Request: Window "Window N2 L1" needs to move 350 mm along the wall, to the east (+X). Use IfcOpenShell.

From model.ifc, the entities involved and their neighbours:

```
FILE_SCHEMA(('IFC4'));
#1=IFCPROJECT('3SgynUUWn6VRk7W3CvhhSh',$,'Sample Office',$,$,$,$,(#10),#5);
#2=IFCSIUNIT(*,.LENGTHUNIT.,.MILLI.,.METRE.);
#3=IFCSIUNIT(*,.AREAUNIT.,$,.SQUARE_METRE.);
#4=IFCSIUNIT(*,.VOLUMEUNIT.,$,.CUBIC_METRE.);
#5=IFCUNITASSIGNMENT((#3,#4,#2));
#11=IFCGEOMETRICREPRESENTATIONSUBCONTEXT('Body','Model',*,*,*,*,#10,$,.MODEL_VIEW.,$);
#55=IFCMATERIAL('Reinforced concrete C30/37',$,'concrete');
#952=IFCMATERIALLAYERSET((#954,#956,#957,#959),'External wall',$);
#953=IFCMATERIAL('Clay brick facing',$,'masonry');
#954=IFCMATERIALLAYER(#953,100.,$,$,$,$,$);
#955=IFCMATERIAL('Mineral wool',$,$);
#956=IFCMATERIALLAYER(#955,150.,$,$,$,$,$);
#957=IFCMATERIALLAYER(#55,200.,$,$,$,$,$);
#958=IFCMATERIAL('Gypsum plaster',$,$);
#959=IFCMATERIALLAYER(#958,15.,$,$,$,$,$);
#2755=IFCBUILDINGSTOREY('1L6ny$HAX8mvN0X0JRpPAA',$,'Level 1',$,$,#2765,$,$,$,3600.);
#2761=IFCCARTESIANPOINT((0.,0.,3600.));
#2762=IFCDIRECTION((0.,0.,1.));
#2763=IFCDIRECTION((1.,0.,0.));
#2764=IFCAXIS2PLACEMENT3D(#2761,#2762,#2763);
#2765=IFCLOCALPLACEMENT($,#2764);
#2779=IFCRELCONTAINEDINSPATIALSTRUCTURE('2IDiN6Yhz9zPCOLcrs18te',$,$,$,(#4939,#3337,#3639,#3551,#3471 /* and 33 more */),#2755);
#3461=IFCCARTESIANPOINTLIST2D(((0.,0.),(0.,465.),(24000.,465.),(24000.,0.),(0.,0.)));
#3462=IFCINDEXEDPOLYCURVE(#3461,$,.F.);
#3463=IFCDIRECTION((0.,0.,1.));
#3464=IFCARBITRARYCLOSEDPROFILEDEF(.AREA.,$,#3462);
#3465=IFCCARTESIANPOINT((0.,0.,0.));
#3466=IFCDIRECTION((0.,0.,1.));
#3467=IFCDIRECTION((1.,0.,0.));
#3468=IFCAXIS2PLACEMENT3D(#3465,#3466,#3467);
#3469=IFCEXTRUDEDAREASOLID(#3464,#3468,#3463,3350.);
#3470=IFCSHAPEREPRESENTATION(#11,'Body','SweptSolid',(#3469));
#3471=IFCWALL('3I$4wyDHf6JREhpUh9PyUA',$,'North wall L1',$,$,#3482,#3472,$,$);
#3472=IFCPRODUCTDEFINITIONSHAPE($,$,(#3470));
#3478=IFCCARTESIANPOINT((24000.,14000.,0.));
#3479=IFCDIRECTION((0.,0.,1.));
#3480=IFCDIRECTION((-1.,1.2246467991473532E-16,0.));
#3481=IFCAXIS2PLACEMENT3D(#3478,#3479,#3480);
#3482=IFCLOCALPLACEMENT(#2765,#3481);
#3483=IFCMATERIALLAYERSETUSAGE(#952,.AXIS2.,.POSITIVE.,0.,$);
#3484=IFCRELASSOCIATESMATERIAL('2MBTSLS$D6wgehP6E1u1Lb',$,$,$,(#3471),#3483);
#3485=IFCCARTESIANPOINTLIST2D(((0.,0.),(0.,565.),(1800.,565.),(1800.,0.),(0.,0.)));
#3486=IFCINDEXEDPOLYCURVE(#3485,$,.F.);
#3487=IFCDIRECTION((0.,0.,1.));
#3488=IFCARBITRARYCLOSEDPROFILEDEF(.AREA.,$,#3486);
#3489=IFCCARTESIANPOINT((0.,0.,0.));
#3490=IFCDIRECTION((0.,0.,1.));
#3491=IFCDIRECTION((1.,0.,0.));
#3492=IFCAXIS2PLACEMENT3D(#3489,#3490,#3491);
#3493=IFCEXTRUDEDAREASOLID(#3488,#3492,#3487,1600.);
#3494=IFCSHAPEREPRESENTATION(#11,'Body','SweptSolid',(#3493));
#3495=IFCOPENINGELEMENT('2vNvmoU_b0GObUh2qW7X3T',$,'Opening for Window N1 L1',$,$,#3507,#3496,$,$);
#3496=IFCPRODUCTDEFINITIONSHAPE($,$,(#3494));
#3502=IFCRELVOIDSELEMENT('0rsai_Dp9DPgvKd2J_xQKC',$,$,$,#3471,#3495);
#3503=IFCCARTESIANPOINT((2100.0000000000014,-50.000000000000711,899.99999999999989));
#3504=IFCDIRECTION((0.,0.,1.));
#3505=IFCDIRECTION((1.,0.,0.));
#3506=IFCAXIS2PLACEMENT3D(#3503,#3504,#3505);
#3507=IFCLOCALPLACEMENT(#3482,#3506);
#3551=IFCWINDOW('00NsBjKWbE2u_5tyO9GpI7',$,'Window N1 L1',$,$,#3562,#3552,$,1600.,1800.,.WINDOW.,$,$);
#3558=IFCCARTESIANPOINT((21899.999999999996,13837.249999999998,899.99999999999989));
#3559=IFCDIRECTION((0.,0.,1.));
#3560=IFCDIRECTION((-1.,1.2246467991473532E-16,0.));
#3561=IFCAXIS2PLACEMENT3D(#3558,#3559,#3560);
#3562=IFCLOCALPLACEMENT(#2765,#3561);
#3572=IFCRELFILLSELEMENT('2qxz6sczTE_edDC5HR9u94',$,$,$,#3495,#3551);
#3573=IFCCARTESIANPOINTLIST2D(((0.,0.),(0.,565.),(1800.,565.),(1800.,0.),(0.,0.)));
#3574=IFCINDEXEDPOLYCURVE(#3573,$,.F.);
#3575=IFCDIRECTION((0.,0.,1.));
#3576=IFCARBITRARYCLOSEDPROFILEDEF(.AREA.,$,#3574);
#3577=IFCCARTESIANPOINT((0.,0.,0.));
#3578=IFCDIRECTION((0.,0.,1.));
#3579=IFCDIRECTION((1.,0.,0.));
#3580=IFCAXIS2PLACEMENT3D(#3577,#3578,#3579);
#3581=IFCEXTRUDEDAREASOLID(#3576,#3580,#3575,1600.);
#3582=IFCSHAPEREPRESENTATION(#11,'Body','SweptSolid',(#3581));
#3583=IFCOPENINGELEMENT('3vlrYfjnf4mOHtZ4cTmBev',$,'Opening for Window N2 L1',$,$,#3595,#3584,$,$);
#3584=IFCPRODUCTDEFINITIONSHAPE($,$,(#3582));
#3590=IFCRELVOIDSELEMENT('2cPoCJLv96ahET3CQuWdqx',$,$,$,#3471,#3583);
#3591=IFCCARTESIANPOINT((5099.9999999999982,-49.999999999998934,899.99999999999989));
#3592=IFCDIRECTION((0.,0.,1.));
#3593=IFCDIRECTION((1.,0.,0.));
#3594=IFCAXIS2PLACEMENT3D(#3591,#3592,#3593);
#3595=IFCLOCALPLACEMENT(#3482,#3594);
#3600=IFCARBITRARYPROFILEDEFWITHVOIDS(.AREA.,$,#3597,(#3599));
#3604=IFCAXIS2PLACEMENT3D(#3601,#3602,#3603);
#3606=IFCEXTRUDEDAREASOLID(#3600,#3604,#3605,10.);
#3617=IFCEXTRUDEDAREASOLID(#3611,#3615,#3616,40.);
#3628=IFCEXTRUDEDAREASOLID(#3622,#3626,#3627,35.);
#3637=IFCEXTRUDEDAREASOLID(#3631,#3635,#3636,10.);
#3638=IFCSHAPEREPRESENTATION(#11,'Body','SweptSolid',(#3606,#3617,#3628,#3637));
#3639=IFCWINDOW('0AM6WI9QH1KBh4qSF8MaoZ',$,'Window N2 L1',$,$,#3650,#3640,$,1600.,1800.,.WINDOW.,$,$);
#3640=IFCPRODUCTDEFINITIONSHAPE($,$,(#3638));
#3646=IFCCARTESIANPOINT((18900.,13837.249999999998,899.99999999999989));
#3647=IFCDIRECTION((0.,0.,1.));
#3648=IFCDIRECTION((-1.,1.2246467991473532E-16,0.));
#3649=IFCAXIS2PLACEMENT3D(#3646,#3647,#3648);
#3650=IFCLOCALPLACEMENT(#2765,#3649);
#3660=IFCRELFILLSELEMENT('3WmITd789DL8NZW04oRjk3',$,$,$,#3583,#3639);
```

```python
import ifcopenshell
import ifcopenshell.api.geometry
import ifcopenshell.util.placement
import ifcopenshell.util.unit

model = ifcopenshell.open("model.ifc")
unit_scale = ifcopenshell.util.unit.calculate_unit_scale(model)

window = model.by_guid("0AM6WI9QH1KBh4qSF8MaoZ")
opening = window.FillsVoids[0].RelatingOpeningElement
wall = opening.VoidsElements[0].RelatingBuildingElement

wall_matrix = ifcopenshell.util.placement.get_local_placement(wall.ObjectPlacement)
shift = wall_matrix[:3, 0] * -0.35 / unit_scale
before = ifcopenshell.util.placement.get_local_placement(window.ObjectPlacement)[:3, 3].copy()

# The window is not placed relative to its opening, so move both.
for product in (opening, window):
    matrix = ifcopenshell.util.placement.get_local_placement(product.ObjectPlacement)
    matrix[:3, 3] += shift
    ifcopenshell.api.geometry.edit_object_placement(model, product=product, matrix=matrix, is_si=False)

after = ifcopenshell.util.placement.get_local_placement(window.ObjectPlacement)[:3, 3]
print("window moved by", (after - before).round(3) + 0.0)

model.write("model_edited.ifc")
```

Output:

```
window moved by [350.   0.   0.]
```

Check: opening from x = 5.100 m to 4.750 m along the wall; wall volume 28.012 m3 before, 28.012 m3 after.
